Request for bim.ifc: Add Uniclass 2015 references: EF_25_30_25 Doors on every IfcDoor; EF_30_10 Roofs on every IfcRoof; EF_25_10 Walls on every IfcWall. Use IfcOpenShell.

First a look at what the model holds.

```python
import ifcopenshell

model = ifcopenshell.open("bim.ifc")
print(model.schema)
print("classifications:", [c.Name for c in model.by_type("IfcClassification")])
for ifc_class in ("IfcDoor", "IfcRoof", "IfcStair", "IfcWall", "IfcWindow"):
    print(ifc_class, len(model.by_type(ifc_class)))
```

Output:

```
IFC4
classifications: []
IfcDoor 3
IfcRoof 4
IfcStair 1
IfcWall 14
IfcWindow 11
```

```python
import ifcopenshell
import ifcopenshell.api.classification

model = ifcopenshell.open("bim.ifc")

system = ifcopenshell.api.classification.add_classification(model, classification="Uniclass 2015")

codes = {
    "IfcDoor": ("EF_25_30_25", "Doors"),
    "IfcRoof": ("EF_30_10", "Roofs"),
    "IfcWall": ("EF_25_10", "Walls"),
}
for ifc_class, (code, name) in codes.items():
    products = model.by_type(ifc_class)
    ifcopenshell.api.classification.add_reference(
        model, products=products, classification=system, identification=code, name=name
    )
    print(code, len(products))

model.write("bim_edited.ifc")
```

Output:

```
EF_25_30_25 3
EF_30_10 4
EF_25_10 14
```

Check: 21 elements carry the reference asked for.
